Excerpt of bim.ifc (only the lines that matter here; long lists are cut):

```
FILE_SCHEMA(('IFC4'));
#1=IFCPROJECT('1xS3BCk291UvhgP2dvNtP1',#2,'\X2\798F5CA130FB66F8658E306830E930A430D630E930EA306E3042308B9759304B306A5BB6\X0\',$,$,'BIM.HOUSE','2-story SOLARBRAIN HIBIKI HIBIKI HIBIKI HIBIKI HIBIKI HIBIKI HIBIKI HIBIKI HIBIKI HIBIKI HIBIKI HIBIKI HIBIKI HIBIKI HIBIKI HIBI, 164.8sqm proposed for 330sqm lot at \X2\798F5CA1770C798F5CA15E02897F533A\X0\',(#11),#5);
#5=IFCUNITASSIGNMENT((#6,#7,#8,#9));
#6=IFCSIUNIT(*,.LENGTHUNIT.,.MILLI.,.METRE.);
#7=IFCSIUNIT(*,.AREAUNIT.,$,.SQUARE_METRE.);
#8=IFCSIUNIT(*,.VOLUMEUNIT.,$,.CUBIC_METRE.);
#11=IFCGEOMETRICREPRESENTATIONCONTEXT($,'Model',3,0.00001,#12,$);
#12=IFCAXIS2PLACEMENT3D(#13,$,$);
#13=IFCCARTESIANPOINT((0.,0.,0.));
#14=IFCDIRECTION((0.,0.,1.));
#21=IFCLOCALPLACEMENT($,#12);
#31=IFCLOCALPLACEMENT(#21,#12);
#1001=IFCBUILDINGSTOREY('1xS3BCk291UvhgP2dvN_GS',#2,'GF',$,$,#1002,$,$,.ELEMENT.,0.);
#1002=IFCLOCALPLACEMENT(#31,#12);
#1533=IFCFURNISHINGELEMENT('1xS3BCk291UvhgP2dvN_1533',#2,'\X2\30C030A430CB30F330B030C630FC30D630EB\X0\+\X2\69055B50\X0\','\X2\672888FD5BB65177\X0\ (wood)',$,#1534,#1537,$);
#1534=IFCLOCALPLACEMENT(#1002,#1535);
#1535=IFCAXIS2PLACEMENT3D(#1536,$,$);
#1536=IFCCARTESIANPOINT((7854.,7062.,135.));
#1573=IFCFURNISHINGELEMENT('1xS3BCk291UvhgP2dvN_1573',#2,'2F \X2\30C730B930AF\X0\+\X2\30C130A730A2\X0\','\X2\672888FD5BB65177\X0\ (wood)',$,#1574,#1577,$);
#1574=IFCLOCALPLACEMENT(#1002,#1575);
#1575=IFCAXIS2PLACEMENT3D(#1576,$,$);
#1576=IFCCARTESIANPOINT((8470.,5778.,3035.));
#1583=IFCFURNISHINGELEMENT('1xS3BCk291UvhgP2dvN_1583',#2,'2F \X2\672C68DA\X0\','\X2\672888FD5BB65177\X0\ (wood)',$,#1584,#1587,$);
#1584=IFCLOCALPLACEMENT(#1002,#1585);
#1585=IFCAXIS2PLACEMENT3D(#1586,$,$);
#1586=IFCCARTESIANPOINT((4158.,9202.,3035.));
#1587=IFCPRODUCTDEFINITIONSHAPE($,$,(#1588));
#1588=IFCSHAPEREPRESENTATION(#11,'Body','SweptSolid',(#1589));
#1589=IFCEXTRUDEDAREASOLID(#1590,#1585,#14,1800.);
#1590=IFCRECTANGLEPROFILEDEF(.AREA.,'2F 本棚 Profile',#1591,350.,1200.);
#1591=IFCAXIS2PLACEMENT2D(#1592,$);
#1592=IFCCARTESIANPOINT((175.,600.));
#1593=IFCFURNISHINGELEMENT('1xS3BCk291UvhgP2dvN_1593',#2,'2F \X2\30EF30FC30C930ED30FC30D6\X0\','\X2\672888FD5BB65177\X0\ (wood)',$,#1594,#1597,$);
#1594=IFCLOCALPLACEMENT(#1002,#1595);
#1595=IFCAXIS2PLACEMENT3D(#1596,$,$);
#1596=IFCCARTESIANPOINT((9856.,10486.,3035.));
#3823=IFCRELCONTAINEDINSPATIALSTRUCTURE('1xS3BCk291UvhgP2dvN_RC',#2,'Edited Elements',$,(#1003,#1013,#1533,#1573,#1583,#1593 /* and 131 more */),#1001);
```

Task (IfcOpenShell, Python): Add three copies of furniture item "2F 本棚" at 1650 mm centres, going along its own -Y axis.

```python
import ifcopenshell
import ifcopenshell.api.geometry
import ifcopenshell.api.root
import ifcopenshell.util.element
import ifcopenshell.util.placement
import ifcopenshell.util.unit

model = ifcopenshell.open("bim.ifc")
unit_scale = ifcopenshell.util.unit.calculate_unit_scale(model)


def reuse_history(source, copy):
    """copy_class also copies each property set's owner history, people and application; keep the originals."""
    for rel in copy.IsDefinedBy:
        if rel.is_a("IfcRelDefinesByProperties") and (history := rel.RelatingPropertyDefinition.OwnerHistory):
            rel.RelatingPropertyDefinition.OwnerHistory = source.OwnerHistory
            ifcopenshell.util.element.remove_deep2(model, history)


source = model.by_guid("1xS3BCk291UvhgP2dvN_1583")
base = ifcopenshell.util.placement.get_local_placement(source.ObjectPlacement)
step = -base[:3, 1] * 1.65 / unit_scale

for i in range(1, 4):
    copy = ifcopenshell.api.root.copy_class(model, product=source)
    copy.Representation = ifcopenshell.util.element.copy_deep(
        model, source.Representation, exclude=["IfcGeometricRepresentationContext", "IfcRepresentationMap"]
    )
    reuse_history(source, copy)
    matrix = base.copy()
    matrix[:3, 3] += i * step
    print("added at", matrix[:3, 3].round(3) + 0.0)
    ifcopenshell.api.geometry.edit_object_placement(model, product=copy, matrix=matrix, is_si=False)

model.write("bim-out.ifc")
```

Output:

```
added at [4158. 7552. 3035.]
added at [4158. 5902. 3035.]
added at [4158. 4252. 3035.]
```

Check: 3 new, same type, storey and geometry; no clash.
